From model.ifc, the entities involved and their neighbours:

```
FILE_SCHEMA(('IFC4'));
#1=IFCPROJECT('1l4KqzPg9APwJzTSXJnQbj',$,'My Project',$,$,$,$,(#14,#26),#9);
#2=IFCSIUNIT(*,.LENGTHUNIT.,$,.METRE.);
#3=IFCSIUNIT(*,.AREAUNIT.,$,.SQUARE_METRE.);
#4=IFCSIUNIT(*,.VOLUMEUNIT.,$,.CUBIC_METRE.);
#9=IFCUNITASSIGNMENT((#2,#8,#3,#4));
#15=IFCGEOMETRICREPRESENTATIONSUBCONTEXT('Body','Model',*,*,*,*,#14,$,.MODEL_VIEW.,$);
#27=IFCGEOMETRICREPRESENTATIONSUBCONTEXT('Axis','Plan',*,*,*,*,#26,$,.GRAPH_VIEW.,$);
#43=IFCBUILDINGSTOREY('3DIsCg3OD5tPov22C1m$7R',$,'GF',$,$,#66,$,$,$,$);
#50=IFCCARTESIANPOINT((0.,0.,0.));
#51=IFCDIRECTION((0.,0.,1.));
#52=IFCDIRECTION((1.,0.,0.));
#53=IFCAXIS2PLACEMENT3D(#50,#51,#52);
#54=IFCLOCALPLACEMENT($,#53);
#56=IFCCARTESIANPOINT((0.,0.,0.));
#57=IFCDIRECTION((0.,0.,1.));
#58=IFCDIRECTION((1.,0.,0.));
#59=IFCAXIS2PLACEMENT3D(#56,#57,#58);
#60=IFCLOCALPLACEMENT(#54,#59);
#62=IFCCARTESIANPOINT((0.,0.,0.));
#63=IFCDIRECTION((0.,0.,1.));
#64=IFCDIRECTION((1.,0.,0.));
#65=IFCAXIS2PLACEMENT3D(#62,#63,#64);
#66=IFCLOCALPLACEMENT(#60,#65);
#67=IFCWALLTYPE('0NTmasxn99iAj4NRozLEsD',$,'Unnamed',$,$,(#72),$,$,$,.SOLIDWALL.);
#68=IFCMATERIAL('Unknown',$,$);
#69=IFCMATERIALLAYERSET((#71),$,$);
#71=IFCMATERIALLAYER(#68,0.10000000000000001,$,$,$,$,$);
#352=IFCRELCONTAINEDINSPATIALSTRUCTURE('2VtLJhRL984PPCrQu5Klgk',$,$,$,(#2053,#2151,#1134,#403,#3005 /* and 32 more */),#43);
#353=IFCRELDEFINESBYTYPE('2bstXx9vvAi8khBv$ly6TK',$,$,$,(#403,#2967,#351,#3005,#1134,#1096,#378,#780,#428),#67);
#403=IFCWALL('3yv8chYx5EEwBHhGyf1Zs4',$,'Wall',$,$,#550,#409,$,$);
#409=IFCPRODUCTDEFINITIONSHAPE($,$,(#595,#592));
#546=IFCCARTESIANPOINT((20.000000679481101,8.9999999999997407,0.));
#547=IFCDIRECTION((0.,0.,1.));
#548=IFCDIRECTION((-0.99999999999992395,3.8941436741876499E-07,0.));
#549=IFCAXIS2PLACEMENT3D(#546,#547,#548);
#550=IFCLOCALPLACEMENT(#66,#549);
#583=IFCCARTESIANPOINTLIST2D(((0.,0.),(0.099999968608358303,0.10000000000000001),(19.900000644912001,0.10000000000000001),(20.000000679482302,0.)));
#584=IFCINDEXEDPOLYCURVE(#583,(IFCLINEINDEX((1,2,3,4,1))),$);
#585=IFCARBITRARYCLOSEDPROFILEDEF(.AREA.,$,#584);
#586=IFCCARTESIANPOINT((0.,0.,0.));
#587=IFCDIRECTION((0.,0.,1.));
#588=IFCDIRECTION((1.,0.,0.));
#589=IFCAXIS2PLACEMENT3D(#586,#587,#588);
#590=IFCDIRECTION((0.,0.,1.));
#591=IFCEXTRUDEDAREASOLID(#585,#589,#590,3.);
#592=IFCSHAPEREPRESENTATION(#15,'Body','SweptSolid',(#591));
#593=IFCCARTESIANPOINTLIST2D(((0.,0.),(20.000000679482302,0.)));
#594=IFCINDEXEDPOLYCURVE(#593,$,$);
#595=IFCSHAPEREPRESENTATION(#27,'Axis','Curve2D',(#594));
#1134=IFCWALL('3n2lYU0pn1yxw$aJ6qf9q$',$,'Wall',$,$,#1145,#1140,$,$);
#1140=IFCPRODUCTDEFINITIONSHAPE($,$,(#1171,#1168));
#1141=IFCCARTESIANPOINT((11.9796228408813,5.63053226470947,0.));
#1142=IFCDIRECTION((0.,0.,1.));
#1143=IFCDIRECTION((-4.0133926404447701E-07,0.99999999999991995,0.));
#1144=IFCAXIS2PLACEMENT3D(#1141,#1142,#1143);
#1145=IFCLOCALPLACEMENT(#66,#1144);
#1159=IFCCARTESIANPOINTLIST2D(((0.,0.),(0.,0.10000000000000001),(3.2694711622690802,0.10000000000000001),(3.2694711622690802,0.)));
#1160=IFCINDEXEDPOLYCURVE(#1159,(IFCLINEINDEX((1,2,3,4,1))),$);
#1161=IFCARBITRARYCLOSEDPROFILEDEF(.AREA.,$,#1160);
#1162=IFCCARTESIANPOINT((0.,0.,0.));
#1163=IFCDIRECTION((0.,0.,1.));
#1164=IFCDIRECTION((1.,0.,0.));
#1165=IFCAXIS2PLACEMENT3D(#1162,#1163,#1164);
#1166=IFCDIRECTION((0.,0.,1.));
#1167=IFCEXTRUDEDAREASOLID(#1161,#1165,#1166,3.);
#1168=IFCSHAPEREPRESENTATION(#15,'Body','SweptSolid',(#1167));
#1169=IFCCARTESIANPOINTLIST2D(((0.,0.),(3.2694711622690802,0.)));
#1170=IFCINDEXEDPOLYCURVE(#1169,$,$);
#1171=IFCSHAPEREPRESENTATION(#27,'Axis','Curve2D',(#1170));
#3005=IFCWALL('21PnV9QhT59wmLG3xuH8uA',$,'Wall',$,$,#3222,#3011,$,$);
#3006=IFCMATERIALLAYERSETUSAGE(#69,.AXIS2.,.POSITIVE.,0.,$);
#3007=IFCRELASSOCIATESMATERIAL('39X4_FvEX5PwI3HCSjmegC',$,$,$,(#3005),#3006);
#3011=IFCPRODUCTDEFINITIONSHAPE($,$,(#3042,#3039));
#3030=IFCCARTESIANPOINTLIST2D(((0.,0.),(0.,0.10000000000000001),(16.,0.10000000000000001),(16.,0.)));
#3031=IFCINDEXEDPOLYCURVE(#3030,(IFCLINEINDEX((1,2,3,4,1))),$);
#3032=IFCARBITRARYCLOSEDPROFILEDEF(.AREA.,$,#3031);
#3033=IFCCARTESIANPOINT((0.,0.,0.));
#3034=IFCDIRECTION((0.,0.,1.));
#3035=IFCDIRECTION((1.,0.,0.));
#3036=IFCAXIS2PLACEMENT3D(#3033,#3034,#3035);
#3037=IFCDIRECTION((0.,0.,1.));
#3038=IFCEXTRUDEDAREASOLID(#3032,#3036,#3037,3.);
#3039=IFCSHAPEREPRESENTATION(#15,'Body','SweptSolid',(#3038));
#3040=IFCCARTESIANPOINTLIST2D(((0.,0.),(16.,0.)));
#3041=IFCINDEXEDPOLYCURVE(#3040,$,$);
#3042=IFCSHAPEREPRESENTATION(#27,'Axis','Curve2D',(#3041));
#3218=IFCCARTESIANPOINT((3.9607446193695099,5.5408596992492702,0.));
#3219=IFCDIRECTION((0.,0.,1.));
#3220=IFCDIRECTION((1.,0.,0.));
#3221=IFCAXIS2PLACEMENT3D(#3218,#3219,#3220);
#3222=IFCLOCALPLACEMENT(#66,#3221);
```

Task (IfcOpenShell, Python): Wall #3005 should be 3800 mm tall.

```python
import ifcopenshell
import ifcopenshell.geom
import ifcopenshell.util.representation
import ifcopenshell.util.shape
import ifcopenshell.util.unit

model = ifcopenshell.open("model.ifc")
unit_scale = ifcopenshell.util.unit.calculate_unit_scale(model)
settings = ifcopenshell.geom.settings()


def volume(element):
    """Net volume in cubic metres, openings subtracted."""
    shape = ifcopenshell.geom.create_shape(settings, element)
    return ifcopenshell.util.shape.get_volume(shape.geometry)


wall = model.by_guid("21PnV9QhT59wmLG3xuH8uA")
before = volume(wall)

body = ifcopenshell.util.representation.get_representation(wall, "Model", "Body")
solid = body.Items[0]
old_height = solid.Depth
solid.Depth = 3.8 / unit_scale
after = volume(wall)

print(f"height {old_height:g} -> {solid.Depth:g}, volume {before:.3f} -> {after:.3f} m3")

model.write("model_v2.ifc")
```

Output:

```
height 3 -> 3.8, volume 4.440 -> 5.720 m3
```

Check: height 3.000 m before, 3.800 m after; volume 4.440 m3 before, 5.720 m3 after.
